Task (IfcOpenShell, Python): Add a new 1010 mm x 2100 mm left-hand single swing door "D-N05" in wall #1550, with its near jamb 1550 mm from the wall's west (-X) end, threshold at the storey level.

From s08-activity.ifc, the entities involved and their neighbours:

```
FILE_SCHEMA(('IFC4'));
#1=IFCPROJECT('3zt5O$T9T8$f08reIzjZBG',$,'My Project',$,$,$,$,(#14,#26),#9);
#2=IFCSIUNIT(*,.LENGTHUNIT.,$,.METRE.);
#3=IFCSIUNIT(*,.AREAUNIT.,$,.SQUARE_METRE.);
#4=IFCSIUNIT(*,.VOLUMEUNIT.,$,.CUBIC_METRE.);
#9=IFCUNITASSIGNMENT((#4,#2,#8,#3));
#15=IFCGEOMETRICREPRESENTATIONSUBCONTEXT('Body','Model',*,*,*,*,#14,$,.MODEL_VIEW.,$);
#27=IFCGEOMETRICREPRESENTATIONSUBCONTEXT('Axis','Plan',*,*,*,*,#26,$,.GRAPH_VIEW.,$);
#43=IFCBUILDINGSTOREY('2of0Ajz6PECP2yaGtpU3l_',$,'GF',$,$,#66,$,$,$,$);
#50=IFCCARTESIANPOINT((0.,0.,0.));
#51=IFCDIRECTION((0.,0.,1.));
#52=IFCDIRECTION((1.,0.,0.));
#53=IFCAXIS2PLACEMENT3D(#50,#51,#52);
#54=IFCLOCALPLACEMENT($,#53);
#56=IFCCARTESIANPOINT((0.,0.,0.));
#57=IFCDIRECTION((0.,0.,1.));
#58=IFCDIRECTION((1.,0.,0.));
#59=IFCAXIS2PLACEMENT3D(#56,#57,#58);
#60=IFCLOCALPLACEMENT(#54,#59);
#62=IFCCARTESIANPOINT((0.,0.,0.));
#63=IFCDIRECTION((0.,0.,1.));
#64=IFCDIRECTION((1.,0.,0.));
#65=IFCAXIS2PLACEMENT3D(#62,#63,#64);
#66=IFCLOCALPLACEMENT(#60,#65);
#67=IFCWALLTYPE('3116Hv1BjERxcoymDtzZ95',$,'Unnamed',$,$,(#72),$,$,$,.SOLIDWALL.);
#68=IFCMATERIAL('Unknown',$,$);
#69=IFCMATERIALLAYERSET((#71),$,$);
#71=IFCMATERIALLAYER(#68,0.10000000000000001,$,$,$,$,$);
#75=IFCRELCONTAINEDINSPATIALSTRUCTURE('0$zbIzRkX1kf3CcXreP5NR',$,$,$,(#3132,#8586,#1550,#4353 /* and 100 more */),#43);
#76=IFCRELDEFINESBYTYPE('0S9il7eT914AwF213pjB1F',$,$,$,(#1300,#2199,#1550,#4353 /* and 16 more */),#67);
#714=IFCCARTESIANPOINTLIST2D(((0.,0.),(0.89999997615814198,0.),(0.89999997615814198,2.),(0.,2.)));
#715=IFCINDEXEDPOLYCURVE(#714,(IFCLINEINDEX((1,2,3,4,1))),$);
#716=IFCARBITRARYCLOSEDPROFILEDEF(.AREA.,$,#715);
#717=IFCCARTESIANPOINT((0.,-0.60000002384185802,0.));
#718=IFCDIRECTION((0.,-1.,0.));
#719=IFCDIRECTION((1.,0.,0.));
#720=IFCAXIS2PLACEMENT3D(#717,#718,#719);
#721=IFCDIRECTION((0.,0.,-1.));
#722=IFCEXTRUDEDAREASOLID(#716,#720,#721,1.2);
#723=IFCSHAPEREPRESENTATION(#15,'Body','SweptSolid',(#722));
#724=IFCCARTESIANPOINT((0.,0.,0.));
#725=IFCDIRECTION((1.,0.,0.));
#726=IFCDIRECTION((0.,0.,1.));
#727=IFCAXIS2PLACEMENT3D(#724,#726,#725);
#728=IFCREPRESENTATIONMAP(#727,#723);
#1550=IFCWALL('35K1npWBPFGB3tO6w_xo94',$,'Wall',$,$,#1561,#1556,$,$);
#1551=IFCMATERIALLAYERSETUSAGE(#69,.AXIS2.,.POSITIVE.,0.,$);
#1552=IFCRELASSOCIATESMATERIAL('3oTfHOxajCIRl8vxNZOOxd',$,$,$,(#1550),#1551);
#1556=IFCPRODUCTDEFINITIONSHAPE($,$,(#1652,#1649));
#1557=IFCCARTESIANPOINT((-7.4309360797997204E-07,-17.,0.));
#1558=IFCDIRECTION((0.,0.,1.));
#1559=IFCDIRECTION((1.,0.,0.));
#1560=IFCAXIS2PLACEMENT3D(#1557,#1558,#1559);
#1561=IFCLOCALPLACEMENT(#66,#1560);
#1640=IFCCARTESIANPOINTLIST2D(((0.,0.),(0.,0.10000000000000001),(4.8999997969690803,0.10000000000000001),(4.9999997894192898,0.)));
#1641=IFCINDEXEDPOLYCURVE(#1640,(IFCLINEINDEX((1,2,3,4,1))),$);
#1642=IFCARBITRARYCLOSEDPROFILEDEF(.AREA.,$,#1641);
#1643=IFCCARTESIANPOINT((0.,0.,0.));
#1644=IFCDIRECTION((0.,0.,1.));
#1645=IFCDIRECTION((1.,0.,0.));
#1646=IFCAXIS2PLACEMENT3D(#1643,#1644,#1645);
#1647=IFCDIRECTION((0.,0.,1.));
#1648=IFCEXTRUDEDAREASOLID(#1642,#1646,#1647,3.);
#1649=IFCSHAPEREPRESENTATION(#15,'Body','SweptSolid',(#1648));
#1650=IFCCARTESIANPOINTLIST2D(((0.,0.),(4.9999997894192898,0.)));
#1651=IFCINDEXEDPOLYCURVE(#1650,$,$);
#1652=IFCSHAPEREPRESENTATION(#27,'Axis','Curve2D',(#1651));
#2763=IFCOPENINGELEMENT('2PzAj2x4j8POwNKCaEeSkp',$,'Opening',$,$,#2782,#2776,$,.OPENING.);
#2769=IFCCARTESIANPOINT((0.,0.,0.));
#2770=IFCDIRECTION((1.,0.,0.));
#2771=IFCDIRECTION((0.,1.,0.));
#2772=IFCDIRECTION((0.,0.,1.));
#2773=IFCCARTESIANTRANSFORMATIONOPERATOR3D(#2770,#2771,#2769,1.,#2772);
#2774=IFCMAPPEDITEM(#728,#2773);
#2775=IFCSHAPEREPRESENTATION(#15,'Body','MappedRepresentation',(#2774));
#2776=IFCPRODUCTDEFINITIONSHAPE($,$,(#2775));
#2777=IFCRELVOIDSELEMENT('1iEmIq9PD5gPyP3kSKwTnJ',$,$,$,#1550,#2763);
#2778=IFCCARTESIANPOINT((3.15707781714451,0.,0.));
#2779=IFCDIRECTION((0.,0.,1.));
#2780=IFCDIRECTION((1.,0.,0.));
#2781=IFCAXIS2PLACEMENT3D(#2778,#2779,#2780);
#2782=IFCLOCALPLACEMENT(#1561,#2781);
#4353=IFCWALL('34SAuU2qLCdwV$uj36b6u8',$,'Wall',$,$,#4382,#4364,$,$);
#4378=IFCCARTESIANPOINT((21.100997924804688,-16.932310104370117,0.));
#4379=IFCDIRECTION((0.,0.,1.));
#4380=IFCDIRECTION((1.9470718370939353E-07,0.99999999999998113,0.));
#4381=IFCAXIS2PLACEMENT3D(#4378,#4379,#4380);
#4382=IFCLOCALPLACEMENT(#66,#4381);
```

```python
import numpy as np
import ifcopenshell
import ifcopenshell.api.feature
import ifcopenshell.api.geometry
import ifcopenshell.api.root
import ifcopenshell.api.spatial
import ifcopenshell.geom
import ifcopenshell.util.element
import ifcopenshell.util.placement
import ifcopenshell.util.representation
import ifcopenshell.util.shape
import ifcopenshell.util.unit

model = ifcopenshell.open("s08-activity.ifc")
unit_scale = ifcopenshell.util.unit.calculate_unit_scale(model)
settings = ifcopenshell.geom.settings()


def volume(element):
    """Net volume in cubic metres, openings subtracted."""
    shape = ifcopenshell.geom.create_shape(settings, element)
    return ifcopenshell.util.shape.get_volume(shape.geometry)


wall = model.by_guid("35K1npWBPFGB3tO6w_xo94")
storey = ifcopenshell.util.element.get_container(wall, ifc_class="IfcBuildingStorey")
context = ifcopenshell.util.representation.get_context(model, "Model", "Body", "MODEL_VIEW")
before = volume(wall)

width, height, from_end, sill = 1.01, 2.1, 1.55, 0.0  # metres

# The wall runs along its own X axis, and the end named is its -X end.
wall_shape = ifcopenshell.geom.create_shape(settings, wall)
x, y, z = ifcopenshell.util.shape.get_vertices(wall_shape.geometry).T
start = x.min() + from_end
face, thickness = float(y.min()), float(y.max() - y.min())
wall_matrix = ifcopenshell.util.placement.get_local_placement(wall.ObjectPlacement)
level = ifcopenshell.util.placement.get_local_placement(storey.ObjectPlacement)[2, 3]


def in_wall(x, y):
    """Placement at x, y metres in the wall's axes, at sill height."""
    matrix = wall_matrix.copy()
    matrix[:, 3] = wall_matrix @ np.array([x / unit_scale, y / unit_scale, 0.0, 1.0])
    matrix[2, 3] = level + sill / unit_scale
    return matrix


# Opening: a box that overshoots both wall faces by 50 mm.
opening = ifcopenshell.api.root.create_entity(model, ifc_class="IfcOpeningElement", predefined_type="OPENING")
box = ifcopenshell.api.geometry.add_wall_representation(
    model, context=context, length=width, height=height, thickness=thickness + 0.1
)
ifcopenshell.api.geometry.assign_representation(model, product=opening, representation=box)
ifcopenshell.api.geometry.edit_object_placement(model, product=opening, matrix=in_wall(start, face - 0.05), is_si=False)
ifcopenshell.api.feature.add_feature(model, feature=opening, element=wall)

door = ifcopenshell.api.root.create_entity(model, ifc_class="IfcDoor", name="D-N05", predefined_type="DOOR")
door.OverallWidth, door.OverallHeight = width / unit_scale, height / unit_scale
door.OperationType = "SINGLE_SWING_LEFT"
body = ifcopenshell.api.geometry.add_door_representation(
    model,
    context=context,
    overall_width=door.OverallWidth,
    overall_height=door.OverallHeight,
    operation_type="SINGLE_SWING_LEFT",
    lining_properties={"LiningDepth": thickness / unit_scale, "ThresholdDepth": thickness / unit_scale},
)
ifcopenshell.api.geometry.assign_representation(model, product=door, representation=body)
ifcopenshell.api.spatial.assign_container(model, products=[door], relating_structure=storey)
ifcopenshell.api.feature.add_filling(model, opening=opening, element=door)

# The lining spans the wall, so the door starts at the wall face.
ifcopenshell.api.geometry.edit_object_placement(model, product=door, matrix=in_wall(start, face), is_si=False)

after = volume(wall)

print(f"wall volume {before:.3f} -> {after:.3f} m3")

model.write("s08-activity-out.ifc")
```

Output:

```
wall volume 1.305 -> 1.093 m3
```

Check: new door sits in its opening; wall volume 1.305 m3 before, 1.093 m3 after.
